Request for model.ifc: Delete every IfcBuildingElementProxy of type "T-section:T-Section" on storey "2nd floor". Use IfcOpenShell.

First a look at what the model holds.

```python
import ifcopenshell
import ifcopenshell.util.element

model = ifcopenshell.open("model.ifc")
print(model.schema)
storey = next(s for s in model.by_type("IfcBuildingStorey") if s.Name == "2nd floor")
proxies = [e for e in ifcopenshell.util.element.get_decomposition(storey) if e.is_a("IfcBuildingElementProxy")]
seen = {}
for e in proxies:
    element_type = ifcopenshell.util.element.get_type(e)
    name = element_type.Name if element_type not in (None, e) else None
    seen[name] = seen.get(name, 0) + 1
for name, count in sorted(seen.items(), key=str):
    print(count, "x", name)
```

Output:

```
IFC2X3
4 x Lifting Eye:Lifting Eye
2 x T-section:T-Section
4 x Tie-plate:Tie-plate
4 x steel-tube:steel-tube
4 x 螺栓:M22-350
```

```python
import ifcopenshell
import ifcopenshell.api.root
import ifcopenshell.util.element

model = ifcopenshell.open("model.ifc")

storey = next(s for s in model.by_type("IfcBuildingStorey") if s.Name == "2nd floor")
proxies = [e for e in ifcopenshell.util.element.get_decomposition(storey) if e.is_a("IfcBuildingElementProxy")]
targets = [e for e in proxies if (t := ifcopenshell.util.element.get_type(e)) not in (None, e) and t.Name == "T-section:T-Section"]

for e in targets:
    ifcopenshell.api.root.remove_product(model, product=e)
print(len(targets), "removed")

model.write("model_v2.ifc")
```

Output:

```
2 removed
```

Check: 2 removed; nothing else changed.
